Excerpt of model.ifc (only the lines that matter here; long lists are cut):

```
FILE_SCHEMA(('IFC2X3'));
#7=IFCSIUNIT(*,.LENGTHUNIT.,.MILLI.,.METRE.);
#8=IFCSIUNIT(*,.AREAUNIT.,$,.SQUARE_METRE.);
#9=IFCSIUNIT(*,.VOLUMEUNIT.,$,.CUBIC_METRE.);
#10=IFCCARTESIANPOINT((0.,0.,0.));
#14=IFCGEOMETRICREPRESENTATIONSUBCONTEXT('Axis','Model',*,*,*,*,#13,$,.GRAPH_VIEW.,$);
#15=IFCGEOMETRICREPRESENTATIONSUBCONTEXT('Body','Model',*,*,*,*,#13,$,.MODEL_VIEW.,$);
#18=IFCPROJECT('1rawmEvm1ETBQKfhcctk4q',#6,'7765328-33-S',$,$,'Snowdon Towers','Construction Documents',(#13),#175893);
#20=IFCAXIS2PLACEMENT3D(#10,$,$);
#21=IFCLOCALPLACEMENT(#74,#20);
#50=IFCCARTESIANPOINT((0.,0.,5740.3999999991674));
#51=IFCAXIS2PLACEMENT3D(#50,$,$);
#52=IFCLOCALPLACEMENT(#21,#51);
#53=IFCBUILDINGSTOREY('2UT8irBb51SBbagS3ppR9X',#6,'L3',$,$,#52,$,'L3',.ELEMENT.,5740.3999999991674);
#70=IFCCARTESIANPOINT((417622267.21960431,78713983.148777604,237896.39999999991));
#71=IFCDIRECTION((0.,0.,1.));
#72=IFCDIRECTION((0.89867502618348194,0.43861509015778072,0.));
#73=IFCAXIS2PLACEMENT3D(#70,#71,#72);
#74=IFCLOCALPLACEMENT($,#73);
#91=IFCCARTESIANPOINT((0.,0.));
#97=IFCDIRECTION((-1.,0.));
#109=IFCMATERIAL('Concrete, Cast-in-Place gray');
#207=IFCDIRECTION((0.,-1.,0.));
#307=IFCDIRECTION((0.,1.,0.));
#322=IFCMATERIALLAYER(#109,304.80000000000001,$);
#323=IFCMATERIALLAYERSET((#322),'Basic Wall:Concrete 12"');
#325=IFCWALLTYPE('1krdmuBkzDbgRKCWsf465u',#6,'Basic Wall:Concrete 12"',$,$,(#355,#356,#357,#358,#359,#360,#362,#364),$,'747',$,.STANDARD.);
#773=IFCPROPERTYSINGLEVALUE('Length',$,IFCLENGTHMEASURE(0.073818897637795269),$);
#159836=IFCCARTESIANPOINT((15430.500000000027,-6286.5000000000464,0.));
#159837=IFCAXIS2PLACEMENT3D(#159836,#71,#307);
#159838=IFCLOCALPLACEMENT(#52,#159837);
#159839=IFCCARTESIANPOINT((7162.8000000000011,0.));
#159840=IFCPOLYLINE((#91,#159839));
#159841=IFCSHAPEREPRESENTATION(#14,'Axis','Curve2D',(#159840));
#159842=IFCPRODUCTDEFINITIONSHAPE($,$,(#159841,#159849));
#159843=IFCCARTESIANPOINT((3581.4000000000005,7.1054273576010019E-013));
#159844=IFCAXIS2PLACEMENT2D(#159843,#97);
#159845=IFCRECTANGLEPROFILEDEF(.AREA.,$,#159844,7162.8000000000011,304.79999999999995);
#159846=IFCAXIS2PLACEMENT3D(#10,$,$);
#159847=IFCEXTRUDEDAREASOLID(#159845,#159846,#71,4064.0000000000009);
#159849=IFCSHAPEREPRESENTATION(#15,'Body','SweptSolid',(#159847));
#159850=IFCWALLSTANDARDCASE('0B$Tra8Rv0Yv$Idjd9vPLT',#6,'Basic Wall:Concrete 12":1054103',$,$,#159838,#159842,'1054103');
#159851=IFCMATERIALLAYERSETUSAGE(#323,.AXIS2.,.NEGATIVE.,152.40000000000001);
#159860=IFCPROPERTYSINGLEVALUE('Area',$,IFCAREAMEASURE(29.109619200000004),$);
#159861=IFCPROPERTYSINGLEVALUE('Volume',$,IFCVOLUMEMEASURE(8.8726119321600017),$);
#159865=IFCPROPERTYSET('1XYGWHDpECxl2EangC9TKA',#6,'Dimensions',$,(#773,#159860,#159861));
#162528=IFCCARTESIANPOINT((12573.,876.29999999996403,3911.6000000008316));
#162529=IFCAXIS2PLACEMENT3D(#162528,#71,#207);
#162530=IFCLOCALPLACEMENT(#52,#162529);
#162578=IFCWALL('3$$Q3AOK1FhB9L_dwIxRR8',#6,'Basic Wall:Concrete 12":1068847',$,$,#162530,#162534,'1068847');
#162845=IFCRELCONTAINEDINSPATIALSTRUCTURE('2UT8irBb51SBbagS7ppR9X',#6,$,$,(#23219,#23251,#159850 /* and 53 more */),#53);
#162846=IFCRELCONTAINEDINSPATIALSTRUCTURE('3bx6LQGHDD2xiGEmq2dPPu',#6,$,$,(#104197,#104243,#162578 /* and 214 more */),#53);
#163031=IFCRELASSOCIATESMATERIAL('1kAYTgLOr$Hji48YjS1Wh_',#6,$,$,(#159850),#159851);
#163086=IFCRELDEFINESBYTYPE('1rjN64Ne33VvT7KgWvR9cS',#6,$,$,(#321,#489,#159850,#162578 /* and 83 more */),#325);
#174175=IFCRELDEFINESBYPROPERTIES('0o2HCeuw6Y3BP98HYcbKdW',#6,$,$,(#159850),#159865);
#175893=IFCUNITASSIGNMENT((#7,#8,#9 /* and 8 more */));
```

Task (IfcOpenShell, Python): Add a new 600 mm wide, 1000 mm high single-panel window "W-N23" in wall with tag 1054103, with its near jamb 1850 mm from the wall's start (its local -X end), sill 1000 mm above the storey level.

```python
import numpy as np
import ifcopenshell
import ifcopenshell.api.feature
import ifcopenshell.api.geometry
import ifcopenshell.api.pset
import ifcopenshell.api.root
import ifcopenshell.api.spatial
import ifcopenshell.api.type
import ifcopenshell.geom
import ifcopenshell.util.element
import ifcopenshell.util.placement
import ifcopenshell.util.representation
import ifcopenshell.util.shape
import ifcopenshell.util.unit

model = ifcopenshell.open("model.ifc")
unit_scale = ifcopenshell.util.unit.calculate_unit_scale(model)
area_scale = ifcopenshell.util.unit.calculate_unit_scale(model, "AREAUNIT")
volume_scale = ifcopenshell.util.unit.calculate_unit_scale(model, "VOLUMEUNIT")
settings = ifcopenshell.geom.settings()


def volume(element):
    """Net volume in cubic metres, openings subtracted."""
    shape = ifcopenshell.geom.create_shape(settings, element)
    return ifcopenshell.util.shape.get_volume(shape.geometry)


wall = model.by_guid("0B$Tra8Rv0Yv$Idjd9vPLT")
storey = ifcopenshell.util.element.get_container(wall, ifc_class="IfcBuildingStorey")
context = ifcopenshell.util.representation.get_context(model, "Model", "Body", "MODEL_VIEW")
before = volume(wall)

width, height, from_end, sill = 0.6, 1, 1.85, 1  # metres

# The wall runs along its own X axis, and the end named is its -X end.
wall_shape = ifcopenshell.geom.create_shape(settings, wall)
x, y, z = ifcopenshell.util.shape.get_vertices(wall_shape.geometry).T
start = x.min() + from_end
face, thickness = float(y.min()), float(y.max() - y.min())
wall_matrix = ifcopenshell.util.placement.get_local_placement(wall.ObjectPlacement)
level = ifcopenshell.util.placement.get_local_placement(storey.ObjectPlacement)[2, 3]


def in_wall(x, y):
    """Placement at x, y metres in the wall's axes, at sill height."""
    matrix = wall_matrix.copy()
    matrix[:, 3] = wall_matrix @ np.array([x / unit_scale, y / unit_scale, 0.0, 1.0])
    matrix[2, 3] = level + sill / unit_scale
    return matrix


# Opening: a box that overshoots both wall faces by 50 mm.
opening = ifcopenshell.api.root.create_entity(model, ifc_class="IfcOpeningElement")
box = ifcopenshell.api.geometry.add_wall_representation(
    model, context=context, length=width, height=height, thickness=thickness + 0.1
)
ifcopenshell.api.geometry.assign_representation(model, product=opening, representation=box)
ifcopenshell.api.geometry.edit_object_placement(model, product=opening, matrix=in_wall(start, face - 0.05), is_si=False)
ifcopenshell.api.feature.add_feature(model, feature=opening, element=wall)

window = ifcopenshell.api.root.create_entity(model, ifc_class="IfcWindow", name="W-N23")
window.OverallWidth, window.OverallHeight = width / unit_scale, height / unit_scale
body = ifcopenshell.api.geometry.add_window_representation(
    model,
    context=context,
    overall_width=window.OverallWidth,
    overall_height=window.OverallHeight,
    partition_type="SINGLE_PANEL",
)
ifcopenshell.api.geometry.assign_representation(model, product=window, representation=body)
ifcopenshell.api.spatial.assign_container(model, products=[window], relating_structure=storey)
fills = ifcopenshell.api.feature.add_filling(model, opening=opening, element=window)
fills.OwnerHistory = window.OwnerHistory  # required in IFC2X3

# IFC2X3 keeps the operation on the window style.
style = ifcopenshell.api.root.create_entity(model, ifc_class="IfcWindowStyle", name="W-N23")
style.OperationType, style.ConstructionType = "SINGLE_PANEL", "NOTDEFINED"
style.ParameterTakesPrecedence = style.Sizeable = False
ifcopenshell.api.type.assign_type(model, related_objects=[window], relating_type=style)

# Centre the window in the wall's thickness.
ifcopenshell.api.geometry.edit_object_placement(model, product=window, matrix=in_wall(start, face), is_si=False)
window_shape = ifcopenshell.geom.create_shape(settings, window)
depth = ifcopenshell.util.shape.get_vertices(window_shape.geometry)[:, 1]
offset = face + thickness / 2 - (depth.min() + depth.max()) / 2
ifcopenshell.api.geometry.edit_object_placement(model, product=window, matrix=in_wall(start, offset), is_si=False)

after = volume(wall)

# Update the wall's stored quantities.
pset = model.by_id(ifcopenshell.util.element.get_pset(wall, "Dimensions", should_inherit=False)["id"])
ifcopenshell.api.pset.edit_pset(model, pset=pset, properties={
    "Area": model.create_entity("IfcAreaMeasure", after / thickness / area_scale),
    "Volume": model.create_entity("IfcVolumeMeasure", after / volume_scale),
})

print(f"wall volume {before:.3f} -> {after:.3f} m3")

model.write("model_v2.ifc")
```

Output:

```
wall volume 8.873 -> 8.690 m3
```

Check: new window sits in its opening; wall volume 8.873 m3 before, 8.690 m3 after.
